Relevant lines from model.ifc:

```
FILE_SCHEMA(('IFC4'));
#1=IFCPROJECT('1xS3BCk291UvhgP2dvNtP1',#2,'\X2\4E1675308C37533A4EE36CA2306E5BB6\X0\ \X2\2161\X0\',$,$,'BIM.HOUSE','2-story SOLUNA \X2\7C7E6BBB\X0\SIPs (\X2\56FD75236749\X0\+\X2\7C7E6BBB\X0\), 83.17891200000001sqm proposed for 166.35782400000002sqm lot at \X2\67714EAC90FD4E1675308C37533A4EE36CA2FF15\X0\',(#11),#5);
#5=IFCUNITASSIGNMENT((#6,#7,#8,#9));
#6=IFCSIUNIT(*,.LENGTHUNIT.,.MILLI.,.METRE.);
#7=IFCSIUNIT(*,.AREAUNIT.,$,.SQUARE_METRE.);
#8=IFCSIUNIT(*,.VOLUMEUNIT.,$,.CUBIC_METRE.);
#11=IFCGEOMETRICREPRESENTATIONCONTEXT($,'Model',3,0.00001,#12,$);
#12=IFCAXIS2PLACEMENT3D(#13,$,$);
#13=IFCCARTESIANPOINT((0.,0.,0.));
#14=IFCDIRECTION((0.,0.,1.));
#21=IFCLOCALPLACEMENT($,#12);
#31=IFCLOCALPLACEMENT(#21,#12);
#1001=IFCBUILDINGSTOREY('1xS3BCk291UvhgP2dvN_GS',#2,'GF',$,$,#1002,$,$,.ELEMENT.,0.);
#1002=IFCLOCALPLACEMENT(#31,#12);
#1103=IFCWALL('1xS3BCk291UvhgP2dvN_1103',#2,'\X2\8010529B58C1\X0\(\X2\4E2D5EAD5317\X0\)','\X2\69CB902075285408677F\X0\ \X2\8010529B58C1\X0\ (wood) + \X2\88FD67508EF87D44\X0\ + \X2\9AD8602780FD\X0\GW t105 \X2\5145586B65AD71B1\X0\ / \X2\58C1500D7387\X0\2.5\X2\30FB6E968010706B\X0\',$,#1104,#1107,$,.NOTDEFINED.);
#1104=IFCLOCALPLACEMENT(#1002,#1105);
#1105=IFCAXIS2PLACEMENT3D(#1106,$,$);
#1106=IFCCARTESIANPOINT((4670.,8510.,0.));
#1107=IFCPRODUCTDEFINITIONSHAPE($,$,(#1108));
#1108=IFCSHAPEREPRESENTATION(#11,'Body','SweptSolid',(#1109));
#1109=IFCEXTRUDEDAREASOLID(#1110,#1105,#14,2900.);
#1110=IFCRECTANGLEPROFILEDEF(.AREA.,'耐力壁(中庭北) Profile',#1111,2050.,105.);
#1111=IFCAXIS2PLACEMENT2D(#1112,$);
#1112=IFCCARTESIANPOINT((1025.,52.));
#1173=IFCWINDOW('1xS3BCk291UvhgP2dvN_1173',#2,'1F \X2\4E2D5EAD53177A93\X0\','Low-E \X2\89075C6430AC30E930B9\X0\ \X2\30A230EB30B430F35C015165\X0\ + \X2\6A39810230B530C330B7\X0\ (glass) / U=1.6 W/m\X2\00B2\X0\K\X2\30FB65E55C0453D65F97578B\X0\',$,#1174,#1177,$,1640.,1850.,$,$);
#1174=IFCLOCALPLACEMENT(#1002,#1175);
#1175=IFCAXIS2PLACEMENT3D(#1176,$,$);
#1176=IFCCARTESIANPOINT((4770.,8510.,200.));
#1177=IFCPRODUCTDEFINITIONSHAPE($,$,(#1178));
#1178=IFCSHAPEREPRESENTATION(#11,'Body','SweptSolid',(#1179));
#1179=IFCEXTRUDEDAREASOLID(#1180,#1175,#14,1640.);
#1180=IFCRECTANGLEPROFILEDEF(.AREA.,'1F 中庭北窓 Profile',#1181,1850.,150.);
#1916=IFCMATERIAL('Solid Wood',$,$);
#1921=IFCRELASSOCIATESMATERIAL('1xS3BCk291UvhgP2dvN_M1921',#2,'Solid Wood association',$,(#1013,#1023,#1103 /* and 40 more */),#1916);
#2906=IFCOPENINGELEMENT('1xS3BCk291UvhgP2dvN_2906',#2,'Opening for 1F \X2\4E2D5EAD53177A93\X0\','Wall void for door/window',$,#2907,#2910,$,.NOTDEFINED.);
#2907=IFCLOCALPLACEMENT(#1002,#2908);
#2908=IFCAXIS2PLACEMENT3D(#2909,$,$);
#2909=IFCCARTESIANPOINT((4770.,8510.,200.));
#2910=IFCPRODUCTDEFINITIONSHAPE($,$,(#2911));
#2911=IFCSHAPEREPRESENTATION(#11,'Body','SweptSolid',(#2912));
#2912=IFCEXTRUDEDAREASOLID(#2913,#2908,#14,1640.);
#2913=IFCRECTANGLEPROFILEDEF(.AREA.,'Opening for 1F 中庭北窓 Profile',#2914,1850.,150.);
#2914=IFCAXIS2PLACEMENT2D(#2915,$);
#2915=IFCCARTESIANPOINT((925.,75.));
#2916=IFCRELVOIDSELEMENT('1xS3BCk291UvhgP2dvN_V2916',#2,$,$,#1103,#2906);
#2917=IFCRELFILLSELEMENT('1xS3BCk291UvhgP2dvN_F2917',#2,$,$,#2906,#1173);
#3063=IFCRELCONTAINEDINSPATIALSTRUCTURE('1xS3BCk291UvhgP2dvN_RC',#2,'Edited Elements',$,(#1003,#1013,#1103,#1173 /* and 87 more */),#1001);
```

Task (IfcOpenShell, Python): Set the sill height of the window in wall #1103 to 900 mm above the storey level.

```python
import numpy as np
import ifcopenshell
import ifcopenshell.api.geometry
import ifcopenshell.geom
import ifcopenshell.util.element
import ifcopenshell.util.placement
import ifcopenshell.util.shape
import ifcopenshell.util.unit

model = ifcopenshell.open("model.ifc")
unit_scale = ifcopenshell.util.unit.calculate_unit_scale(model)

window = model.by_guid("1xS3BCk291UvhgP2dvN_1173")
opening = window.FillsVoids[0].RelatingOpeningElement
storey = ifcopenshell.util.element.get_container(window, ifc_class="IfcBuildingStorey")
level = ifcopenshell.util.placement.get_local_placement(storey.ObjectPlacement)[2, 3]

# The opening's origin need not be at the sill, so measure its lowest point.
shape = ifcopenshell.geom.create_shape(ifcopenshell.geom.settings(), opening)
bottom = ifcopenshell.util.shape.get_shape_bottom_elevation(shape, shape.geometry) / unit_scale
dz = level + 900.0 - bottom

shift = np.array([0.0, 0.0, dz])
# The window is not placed relative to its opening, so move both.
for product in (opening, window):
    matrix = ifcopenshell.util.placement.get_local_placement(product.ObjectPlacement)
    matrix[:3, 3] += shift
    ifcopenshell.api.geometry.edit_object_placement(model, product=product, matrix=matrix, is_si=False)

print(f"moved by {dz * unit_scale:+.3f} m")

model.write("model_edited.ifc")
```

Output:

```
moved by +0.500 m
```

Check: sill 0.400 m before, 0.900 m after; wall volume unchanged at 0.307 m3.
